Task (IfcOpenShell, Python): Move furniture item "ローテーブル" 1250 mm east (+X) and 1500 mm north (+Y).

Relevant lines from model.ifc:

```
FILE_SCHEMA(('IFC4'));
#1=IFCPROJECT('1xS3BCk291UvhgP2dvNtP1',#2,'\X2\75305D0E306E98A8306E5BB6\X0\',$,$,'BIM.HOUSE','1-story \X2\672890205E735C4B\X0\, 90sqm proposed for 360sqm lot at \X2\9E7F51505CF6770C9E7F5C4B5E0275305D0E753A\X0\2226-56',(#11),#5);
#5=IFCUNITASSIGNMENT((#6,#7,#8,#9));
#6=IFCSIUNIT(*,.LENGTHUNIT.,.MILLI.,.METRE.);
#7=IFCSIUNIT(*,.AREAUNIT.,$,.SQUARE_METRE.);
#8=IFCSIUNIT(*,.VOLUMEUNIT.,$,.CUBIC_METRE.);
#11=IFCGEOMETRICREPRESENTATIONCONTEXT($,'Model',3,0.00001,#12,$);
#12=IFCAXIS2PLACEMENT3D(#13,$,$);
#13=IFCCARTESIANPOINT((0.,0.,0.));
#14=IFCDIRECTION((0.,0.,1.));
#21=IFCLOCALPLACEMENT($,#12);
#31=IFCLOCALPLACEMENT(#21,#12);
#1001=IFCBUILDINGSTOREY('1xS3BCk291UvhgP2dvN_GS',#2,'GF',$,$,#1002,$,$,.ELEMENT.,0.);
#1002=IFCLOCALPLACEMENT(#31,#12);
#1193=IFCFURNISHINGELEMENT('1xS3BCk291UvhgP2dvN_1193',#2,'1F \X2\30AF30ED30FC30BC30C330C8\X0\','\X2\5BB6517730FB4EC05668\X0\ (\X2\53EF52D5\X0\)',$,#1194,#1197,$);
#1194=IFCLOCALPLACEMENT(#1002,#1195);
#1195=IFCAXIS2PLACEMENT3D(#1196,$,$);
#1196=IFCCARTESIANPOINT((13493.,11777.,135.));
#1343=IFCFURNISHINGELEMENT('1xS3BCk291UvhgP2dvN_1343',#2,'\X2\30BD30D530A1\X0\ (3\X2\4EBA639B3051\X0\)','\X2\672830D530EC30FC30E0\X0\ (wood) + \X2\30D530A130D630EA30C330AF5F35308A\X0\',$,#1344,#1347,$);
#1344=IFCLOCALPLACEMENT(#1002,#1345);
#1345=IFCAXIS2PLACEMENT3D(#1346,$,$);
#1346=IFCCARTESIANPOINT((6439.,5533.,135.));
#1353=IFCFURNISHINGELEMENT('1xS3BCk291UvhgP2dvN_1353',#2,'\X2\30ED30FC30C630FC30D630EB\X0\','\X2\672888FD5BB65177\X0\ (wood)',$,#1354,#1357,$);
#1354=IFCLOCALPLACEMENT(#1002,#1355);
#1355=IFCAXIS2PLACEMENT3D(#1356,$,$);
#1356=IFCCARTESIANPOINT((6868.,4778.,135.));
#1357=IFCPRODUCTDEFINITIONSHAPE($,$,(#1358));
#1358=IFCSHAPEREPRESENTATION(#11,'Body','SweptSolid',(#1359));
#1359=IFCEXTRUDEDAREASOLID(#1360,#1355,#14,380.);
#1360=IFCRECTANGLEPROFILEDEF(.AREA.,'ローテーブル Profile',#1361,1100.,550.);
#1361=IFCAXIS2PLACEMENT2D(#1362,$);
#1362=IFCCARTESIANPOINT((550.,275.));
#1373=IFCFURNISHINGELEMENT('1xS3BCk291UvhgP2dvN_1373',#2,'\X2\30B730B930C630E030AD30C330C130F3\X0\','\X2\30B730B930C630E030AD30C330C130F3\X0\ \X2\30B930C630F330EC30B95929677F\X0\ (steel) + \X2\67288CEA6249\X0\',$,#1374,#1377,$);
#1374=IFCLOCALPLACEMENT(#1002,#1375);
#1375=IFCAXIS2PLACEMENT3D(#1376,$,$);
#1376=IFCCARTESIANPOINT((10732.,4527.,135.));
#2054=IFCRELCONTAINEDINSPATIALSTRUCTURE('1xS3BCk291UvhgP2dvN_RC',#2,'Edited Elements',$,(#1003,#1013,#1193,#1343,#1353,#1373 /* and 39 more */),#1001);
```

```python
import ifcopenshell
import ifcopenshell.api.geometry
import ifcopenshell.util.placement

model = ifcopenshell.open("model.ifc")

item = model.by_guid("1xS3BCk291UvhgP2dvN_1353")
matrix = ifcopenshell.util.placement.get_local_placement(item.ObjectPlacement)
matrix[0, 3] += 1250.0
matrix[1, 3] += 1500.0
ifcopenshell.api.geometry.edit_object_placement(model, product=item, matrix=matrix, is_si=False)

print(ifcopenshell.util.placement.get_local_placement(item.ObjectPlacement).round(3) + 0.0)

model.write("model_updated.ifc")
```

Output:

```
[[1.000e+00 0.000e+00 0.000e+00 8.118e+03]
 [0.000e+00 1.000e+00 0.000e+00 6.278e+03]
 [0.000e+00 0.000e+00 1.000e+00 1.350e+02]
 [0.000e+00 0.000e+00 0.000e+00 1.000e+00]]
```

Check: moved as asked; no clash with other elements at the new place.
